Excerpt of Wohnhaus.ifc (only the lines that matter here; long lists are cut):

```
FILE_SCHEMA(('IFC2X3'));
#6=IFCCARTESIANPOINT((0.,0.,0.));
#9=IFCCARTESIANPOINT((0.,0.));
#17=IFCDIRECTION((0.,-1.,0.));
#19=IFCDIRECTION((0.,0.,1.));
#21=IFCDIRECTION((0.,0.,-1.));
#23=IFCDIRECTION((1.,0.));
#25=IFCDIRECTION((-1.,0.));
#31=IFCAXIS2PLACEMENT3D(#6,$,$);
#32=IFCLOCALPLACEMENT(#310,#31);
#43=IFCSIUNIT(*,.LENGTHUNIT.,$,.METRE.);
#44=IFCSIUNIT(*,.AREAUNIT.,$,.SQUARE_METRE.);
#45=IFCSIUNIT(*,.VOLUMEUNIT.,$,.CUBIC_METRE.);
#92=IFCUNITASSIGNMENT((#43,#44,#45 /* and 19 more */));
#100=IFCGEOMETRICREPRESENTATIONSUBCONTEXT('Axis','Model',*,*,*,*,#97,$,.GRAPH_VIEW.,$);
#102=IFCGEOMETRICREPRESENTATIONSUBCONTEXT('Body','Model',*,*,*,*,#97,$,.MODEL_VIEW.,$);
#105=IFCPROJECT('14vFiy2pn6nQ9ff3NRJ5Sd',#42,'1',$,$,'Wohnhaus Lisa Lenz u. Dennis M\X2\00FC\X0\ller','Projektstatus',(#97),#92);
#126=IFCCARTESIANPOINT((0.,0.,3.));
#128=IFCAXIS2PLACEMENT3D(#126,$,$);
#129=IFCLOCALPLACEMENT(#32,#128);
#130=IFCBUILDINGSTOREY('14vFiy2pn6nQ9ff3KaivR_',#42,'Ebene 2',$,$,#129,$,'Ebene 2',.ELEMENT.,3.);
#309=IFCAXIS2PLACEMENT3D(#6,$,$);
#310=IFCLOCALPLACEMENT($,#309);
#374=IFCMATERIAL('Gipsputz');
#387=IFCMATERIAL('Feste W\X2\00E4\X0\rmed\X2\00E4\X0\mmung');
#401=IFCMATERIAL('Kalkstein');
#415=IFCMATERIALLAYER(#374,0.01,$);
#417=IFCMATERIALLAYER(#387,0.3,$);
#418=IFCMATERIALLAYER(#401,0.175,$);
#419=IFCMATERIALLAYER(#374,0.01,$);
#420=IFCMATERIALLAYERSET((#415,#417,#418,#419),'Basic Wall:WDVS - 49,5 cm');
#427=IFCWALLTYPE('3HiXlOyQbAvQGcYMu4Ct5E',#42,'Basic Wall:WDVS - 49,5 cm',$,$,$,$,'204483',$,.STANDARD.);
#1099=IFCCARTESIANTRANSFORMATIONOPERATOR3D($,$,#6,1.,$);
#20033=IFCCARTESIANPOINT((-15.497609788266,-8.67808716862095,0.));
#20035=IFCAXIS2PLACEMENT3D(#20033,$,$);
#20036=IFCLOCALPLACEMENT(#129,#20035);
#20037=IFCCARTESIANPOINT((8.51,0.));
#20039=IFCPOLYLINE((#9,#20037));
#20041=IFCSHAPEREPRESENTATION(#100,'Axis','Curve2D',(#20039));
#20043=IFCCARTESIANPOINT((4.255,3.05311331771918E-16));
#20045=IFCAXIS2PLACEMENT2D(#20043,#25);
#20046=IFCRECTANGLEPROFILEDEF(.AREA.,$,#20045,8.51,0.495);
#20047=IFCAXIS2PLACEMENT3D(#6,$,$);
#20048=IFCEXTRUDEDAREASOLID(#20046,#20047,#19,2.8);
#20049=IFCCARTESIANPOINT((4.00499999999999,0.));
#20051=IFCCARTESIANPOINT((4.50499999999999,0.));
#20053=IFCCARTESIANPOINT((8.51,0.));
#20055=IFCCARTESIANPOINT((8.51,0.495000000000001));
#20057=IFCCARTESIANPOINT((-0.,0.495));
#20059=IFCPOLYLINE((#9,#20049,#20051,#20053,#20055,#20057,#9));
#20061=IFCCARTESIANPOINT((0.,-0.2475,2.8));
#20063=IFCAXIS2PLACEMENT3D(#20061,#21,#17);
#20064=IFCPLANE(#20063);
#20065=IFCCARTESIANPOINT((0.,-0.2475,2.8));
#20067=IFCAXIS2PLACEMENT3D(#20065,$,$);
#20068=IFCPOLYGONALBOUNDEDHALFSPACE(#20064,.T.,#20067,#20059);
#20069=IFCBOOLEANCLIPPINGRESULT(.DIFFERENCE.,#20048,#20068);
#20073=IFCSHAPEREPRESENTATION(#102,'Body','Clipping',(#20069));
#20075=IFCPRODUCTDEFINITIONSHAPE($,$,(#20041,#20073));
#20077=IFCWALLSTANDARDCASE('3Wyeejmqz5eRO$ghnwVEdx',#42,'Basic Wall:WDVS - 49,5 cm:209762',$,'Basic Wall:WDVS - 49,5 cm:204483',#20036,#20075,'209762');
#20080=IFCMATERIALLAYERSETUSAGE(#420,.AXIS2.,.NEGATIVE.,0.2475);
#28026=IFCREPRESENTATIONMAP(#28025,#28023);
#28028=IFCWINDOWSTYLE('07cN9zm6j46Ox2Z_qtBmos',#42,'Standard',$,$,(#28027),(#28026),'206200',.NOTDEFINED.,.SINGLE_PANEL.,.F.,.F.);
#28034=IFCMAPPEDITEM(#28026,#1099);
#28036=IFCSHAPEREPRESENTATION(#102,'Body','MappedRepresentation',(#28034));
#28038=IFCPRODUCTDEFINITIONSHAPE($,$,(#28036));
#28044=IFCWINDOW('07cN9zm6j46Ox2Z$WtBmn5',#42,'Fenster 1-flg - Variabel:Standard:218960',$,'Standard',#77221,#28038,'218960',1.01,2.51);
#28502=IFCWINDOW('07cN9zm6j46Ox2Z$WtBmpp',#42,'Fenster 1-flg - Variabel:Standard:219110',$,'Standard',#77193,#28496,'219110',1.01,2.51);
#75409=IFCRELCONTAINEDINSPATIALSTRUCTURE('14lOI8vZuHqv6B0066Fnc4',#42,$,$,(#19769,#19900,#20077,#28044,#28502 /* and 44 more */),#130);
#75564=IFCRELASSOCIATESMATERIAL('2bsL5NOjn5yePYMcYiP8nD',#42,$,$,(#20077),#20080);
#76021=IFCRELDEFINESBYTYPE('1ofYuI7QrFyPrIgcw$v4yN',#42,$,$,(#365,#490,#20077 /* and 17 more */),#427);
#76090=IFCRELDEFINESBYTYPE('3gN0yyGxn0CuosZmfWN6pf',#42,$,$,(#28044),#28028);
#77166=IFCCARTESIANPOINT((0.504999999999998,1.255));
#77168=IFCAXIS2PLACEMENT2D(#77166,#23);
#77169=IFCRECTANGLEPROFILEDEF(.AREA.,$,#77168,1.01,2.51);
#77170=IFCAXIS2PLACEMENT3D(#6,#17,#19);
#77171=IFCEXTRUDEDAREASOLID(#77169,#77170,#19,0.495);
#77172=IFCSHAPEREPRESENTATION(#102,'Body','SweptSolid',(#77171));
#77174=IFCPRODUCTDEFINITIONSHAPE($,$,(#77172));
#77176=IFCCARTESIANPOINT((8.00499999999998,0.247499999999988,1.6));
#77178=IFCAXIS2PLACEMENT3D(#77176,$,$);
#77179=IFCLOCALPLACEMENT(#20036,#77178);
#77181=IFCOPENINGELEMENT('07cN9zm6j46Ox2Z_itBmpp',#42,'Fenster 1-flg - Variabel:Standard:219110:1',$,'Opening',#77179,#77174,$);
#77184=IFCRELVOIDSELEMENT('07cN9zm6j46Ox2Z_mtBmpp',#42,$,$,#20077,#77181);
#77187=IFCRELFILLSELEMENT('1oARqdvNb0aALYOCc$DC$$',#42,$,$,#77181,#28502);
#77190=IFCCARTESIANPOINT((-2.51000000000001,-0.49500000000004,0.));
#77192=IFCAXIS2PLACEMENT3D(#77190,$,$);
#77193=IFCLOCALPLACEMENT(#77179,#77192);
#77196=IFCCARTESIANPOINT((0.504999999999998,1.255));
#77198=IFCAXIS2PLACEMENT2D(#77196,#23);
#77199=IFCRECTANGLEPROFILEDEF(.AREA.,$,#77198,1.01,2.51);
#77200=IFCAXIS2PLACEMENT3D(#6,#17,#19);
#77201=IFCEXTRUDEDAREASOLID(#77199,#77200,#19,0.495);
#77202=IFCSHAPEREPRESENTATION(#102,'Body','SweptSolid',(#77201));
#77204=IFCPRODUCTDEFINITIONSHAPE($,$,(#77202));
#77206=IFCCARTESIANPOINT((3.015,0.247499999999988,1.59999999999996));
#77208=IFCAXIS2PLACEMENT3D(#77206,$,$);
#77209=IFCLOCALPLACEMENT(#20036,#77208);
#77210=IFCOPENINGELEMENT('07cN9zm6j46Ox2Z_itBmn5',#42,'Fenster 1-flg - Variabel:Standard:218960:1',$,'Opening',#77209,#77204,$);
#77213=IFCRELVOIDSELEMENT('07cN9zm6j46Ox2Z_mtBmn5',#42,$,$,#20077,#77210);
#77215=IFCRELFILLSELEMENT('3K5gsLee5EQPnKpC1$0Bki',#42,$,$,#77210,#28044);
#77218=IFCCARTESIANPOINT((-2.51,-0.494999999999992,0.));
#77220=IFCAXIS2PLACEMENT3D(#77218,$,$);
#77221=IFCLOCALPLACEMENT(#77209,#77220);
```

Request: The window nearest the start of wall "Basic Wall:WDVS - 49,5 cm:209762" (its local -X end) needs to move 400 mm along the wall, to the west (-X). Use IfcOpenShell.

```python
import ifcopenshell
import ifcopenshell.api.geometry
import ifcopenshell.util.placement
import ifcopenshell.util.unit

model = ifcopenshell.open("Wohnhaus.ifc")
unit_scale = ifcopenshell.util.unit.calculate_unit_scale(model)

window = model.by_guid("07cN9zm6j46Ox2Z$WtBmn5")
opening = window.FillsVoids[0].RelatingOpeningElement
wall = opening.VoidsElements[0].RelatingBuildingElement

wall_matrix = ifcopenshell.util.placement.get_local_placement(wall.ObjectPlacement)
shift = wall_matrix[:3, 0] * -0.4 / unit_scale
before = ifcopenshell.util.placement.get_local_placement(window.ObjectPlacement)[:3, 3].copy()

# The window is placed relative to its opening, so it follows when the opening moves.
matrix = ifcopenshell.util.placement.get_local_placement(opening.ObjectPlacement)
matrix[:3, 3] += shift
ifcopenshell.api.geometry.edit_object_placement(
    model, product=opening, matrix=matrix, is_si=False, should_transform_children=True
)

after = ifcopenshell.util.placement.get_local_placement(window.ObjectPlacement)[:3, 3]
print("window moved by", (after - before).round(3) + 0.0)

model.write("Wohnhaus_rev.ifc")
```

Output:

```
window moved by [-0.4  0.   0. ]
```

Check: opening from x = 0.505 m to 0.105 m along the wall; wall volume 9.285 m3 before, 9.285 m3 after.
